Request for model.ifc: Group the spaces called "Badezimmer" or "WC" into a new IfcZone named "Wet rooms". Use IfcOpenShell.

First a look at what the model holds.

```python
import ifcopenshell

model = ifcopenshell.open("model.ifc")
print(model.schema)
seen = {}
for space in model.by_type("IfcSpace"):
    seen[space.LongName] = seen.get(space.LongName, 0) + 1
for name, count in sorted(seen.items(), key=str):
    print(count, "x", name)
print("zones:", [z.Name for z in model.by_type("IfcZone")][:20])
```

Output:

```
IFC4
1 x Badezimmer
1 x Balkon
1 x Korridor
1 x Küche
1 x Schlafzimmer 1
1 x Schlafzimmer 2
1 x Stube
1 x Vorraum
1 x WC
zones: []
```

```python
import ifcopenshell
import ifcopenshell.api.group
import ifcopenshell.api.root

model = ifcopenshell.open("model.ifc")

names = {"Badezimmer", "WC"}
spaces = [s for s in model.by_type("IfcSpace") if s.LongName in names]

zone = ifcopenshell.api.root.create_entity(model, ifc_class="IfcZone", name="Wet rooms")
ifcopenshell.api.group.assign_group(model, products=spaces, group=zone)
print(len(spaces), "spaces in", zone.Name)

model.write("model_v2.ifc")
```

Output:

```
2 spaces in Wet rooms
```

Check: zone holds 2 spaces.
